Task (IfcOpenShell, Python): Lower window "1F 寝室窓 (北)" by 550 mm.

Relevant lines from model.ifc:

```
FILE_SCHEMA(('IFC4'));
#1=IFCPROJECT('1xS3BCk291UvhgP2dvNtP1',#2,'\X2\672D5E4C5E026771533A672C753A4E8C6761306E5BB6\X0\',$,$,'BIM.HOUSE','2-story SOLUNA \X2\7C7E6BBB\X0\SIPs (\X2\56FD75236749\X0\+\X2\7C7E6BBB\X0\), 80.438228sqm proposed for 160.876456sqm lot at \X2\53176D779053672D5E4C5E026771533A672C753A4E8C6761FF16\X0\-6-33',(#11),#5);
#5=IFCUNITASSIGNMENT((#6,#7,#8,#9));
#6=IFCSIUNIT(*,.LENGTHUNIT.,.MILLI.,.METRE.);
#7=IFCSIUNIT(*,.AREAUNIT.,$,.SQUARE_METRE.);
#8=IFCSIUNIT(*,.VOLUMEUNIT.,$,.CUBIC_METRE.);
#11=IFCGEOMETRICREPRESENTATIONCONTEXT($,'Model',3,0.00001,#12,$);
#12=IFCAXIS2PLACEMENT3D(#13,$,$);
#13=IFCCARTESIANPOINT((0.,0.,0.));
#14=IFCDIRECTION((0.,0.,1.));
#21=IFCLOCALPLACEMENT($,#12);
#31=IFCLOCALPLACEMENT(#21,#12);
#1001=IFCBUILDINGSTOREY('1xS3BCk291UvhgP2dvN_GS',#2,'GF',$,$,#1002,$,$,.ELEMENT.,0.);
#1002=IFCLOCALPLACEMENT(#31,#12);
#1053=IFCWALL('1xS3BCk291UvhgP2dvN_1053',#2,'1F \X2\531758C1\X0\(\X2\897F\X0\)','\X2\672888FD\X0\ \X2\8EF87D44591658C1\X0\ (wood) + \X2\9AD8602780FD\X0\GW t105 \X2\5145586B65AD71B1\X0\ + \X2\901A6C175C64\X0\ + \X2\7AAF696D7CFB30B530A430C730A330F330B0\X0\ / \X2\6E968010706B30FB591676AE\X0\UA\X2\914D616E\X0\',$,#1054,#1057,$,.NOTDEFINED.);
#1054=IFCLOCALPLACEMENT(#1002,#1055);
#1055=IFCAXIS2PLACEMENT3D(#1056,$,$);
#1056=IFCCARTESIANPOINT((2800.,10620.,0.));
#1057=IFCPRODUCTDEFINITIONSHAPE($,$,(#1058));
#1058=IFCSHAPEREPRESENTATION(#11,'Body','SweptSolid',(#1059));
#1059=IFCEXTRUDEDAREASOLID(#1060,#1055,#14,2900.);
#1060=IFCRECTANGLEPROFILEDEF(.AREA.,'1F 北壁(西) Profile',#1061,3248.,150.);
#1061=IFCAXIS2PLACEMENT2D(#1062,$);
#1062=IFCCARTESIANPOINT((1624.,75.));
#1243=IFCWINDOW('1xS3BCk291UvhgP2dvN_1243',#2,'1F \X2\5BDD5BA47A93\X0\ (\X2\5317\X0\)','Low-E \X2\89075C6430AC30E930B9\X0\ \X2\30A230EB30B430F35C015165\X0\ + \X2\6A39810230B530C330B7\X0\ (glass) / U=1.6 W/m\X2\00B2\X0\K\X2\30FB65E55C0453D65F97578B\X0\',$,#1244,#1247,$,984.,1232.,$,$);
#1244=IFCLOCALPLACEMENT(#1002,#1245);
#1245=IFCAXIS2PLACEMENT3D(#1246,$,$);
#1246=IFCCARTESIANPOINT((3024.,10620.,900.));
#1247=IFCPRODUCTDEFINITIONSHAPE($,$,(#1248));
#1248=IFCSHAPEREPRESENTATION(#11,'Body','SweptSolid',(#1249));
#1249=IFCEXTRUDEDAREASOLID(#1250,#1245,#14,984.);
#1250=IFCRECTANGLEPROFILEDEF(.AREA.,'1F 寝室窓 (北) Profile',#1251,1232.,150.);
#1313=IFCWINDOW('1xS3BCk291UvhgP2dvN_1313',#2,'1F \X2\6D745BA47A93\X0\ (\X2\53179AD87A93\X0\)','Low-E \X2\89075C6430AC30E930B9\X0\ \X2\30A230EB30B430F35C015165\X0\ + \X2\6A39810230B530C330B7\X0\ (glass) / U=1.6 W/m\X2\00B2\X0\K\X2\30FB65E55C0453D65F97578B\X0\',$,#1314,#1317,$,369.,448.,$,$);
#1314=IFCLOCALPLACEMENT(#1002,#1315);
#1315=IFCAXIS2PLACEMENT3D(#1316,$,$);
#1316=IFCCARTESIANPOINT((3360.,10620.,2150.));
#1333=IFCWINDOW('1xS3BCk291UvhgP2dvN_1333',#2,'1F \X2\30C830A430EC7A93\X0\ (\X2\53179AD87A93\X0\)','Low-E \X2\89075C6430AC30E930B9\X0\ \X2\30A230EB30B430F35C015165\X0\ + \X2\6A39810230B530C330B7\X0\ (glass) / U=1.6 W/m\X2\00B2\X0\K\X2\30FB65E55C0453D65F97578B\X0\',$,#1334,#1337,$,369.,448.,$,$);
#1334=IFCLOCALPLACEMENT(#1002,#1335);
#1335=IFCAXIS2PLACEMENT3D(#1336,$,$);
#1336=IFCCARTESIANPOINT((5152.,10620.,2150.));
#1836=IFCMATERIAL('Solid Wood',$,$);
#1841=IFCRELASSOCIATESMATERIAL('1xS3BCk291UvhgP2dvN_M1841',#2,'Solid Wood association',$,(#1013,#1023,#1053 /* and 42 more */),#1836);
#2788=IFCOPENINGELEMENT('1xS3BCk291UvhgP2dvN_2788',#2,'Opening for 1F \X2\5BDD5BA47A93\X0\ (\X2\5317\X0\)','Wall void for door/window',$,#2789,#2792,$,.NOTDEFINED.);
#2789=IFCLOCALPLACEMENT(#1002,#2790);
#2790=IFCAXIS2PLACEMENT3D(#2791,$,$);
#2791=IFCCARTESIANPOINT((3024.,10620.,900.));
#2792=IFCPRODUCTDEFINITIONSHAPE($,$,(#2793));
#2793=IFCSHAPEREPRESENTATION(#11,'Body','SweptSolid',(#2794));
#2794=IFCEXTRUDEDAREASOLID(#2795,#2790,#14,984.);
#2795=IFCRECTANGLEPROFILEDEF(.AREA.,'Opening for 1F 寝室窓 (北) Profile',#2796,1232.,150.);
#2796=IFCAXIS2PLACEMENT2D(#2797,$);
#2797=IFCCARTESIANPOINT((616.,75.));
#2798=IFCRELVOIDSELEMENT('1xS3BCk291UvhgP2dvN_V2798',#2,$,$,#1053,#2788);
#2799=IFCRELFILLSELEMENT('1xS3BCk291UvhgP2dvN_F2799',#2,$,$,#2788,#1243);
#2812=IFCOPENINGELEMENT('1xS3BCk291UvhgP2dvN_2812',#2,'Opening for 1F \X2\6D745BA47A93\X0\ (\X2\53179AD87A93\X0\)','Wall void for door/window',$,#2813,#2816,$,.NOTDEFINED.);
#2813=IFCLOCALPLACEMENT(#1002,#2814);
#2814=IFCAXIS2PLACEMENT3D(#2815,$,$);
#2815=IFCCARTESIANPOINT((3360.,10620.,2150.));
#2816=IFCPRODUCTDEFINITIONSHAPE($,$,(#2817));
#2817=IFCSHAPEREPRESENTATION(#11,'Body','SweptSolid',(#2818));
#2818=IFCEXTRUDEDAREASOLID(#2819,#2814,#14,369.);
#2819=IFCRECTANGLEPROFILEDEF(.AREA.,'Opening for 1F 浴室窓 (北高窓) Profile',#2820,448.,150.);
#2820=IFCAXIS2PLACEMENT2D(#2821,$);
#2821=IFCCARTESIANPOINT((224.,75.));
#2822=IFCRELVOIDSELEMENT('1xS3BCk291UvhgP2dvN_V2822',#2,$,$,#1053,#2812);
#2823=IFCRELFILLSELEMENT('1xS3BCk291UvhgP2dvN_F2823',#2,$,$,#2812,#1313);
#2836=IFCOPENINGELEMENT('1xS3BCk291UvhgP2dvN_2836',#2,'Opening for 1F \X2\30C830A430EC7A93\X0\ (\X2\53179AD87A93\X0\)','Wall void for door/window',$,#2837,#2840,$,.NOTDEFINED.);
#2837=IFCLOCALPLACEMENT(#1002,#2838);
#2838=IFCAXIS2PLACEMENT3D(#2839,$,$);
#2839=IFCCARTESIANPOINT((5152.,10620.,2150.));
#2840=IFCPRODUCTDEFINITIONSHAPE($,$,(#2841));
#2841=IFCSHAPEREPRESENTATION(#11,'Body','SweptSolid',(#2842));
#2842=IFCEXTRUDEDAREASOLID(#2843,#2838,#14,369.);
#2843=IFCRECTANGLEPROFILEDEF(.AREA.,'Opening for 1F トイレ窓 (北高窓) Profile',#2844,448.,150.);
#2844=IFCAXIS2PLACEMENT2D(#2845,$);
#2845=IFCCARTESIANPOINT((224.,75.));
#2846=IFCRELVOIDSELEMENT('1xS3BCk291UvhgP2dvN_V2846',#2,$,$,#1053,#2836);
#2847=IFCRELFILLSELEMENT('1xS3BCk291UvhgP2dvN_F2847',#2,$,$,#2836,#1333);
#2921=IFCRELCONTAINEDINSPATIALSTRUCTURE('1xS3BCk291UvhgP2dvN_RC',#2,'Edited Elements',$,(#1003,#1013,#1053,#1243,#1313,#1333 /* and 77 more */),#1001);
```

```python
import numpy as np
import ifcopenshell
import ifcopenshell.api.geometry
import ifcopenshell.util.placement
import ifcopenshell.util.unit

model = ifcopenshell.open("model.ifc")
unit_scale = ifcopenshell.util.unit.calculate_unit_scale(model)

window = model.by_guid("1xS3BCk291UvhgP2dvN_1243")
opening = window.FillsVoids[0].RelatingOpeningElement
dz = -550.0

shift = np.array([0.0, 0.0, dz])
# The window is not placed relative to its opening, so move both.
for product in (opening, window):
    matrix = ifcopenshell.util.placement.get_local_placement(product.ObjectPlacement)
    matrix[:3, 3] += shift
    ifcopenshell.api.geometry.edit_object_placement(model, product=product, matrix=matrix, is_si=False)

print(f"moved by {dz * unit_scale:+.3f} m")

model.write("model-out.ifc")
```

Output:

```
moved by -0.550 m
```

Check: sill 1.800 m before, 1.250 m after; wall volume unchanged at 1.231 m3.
